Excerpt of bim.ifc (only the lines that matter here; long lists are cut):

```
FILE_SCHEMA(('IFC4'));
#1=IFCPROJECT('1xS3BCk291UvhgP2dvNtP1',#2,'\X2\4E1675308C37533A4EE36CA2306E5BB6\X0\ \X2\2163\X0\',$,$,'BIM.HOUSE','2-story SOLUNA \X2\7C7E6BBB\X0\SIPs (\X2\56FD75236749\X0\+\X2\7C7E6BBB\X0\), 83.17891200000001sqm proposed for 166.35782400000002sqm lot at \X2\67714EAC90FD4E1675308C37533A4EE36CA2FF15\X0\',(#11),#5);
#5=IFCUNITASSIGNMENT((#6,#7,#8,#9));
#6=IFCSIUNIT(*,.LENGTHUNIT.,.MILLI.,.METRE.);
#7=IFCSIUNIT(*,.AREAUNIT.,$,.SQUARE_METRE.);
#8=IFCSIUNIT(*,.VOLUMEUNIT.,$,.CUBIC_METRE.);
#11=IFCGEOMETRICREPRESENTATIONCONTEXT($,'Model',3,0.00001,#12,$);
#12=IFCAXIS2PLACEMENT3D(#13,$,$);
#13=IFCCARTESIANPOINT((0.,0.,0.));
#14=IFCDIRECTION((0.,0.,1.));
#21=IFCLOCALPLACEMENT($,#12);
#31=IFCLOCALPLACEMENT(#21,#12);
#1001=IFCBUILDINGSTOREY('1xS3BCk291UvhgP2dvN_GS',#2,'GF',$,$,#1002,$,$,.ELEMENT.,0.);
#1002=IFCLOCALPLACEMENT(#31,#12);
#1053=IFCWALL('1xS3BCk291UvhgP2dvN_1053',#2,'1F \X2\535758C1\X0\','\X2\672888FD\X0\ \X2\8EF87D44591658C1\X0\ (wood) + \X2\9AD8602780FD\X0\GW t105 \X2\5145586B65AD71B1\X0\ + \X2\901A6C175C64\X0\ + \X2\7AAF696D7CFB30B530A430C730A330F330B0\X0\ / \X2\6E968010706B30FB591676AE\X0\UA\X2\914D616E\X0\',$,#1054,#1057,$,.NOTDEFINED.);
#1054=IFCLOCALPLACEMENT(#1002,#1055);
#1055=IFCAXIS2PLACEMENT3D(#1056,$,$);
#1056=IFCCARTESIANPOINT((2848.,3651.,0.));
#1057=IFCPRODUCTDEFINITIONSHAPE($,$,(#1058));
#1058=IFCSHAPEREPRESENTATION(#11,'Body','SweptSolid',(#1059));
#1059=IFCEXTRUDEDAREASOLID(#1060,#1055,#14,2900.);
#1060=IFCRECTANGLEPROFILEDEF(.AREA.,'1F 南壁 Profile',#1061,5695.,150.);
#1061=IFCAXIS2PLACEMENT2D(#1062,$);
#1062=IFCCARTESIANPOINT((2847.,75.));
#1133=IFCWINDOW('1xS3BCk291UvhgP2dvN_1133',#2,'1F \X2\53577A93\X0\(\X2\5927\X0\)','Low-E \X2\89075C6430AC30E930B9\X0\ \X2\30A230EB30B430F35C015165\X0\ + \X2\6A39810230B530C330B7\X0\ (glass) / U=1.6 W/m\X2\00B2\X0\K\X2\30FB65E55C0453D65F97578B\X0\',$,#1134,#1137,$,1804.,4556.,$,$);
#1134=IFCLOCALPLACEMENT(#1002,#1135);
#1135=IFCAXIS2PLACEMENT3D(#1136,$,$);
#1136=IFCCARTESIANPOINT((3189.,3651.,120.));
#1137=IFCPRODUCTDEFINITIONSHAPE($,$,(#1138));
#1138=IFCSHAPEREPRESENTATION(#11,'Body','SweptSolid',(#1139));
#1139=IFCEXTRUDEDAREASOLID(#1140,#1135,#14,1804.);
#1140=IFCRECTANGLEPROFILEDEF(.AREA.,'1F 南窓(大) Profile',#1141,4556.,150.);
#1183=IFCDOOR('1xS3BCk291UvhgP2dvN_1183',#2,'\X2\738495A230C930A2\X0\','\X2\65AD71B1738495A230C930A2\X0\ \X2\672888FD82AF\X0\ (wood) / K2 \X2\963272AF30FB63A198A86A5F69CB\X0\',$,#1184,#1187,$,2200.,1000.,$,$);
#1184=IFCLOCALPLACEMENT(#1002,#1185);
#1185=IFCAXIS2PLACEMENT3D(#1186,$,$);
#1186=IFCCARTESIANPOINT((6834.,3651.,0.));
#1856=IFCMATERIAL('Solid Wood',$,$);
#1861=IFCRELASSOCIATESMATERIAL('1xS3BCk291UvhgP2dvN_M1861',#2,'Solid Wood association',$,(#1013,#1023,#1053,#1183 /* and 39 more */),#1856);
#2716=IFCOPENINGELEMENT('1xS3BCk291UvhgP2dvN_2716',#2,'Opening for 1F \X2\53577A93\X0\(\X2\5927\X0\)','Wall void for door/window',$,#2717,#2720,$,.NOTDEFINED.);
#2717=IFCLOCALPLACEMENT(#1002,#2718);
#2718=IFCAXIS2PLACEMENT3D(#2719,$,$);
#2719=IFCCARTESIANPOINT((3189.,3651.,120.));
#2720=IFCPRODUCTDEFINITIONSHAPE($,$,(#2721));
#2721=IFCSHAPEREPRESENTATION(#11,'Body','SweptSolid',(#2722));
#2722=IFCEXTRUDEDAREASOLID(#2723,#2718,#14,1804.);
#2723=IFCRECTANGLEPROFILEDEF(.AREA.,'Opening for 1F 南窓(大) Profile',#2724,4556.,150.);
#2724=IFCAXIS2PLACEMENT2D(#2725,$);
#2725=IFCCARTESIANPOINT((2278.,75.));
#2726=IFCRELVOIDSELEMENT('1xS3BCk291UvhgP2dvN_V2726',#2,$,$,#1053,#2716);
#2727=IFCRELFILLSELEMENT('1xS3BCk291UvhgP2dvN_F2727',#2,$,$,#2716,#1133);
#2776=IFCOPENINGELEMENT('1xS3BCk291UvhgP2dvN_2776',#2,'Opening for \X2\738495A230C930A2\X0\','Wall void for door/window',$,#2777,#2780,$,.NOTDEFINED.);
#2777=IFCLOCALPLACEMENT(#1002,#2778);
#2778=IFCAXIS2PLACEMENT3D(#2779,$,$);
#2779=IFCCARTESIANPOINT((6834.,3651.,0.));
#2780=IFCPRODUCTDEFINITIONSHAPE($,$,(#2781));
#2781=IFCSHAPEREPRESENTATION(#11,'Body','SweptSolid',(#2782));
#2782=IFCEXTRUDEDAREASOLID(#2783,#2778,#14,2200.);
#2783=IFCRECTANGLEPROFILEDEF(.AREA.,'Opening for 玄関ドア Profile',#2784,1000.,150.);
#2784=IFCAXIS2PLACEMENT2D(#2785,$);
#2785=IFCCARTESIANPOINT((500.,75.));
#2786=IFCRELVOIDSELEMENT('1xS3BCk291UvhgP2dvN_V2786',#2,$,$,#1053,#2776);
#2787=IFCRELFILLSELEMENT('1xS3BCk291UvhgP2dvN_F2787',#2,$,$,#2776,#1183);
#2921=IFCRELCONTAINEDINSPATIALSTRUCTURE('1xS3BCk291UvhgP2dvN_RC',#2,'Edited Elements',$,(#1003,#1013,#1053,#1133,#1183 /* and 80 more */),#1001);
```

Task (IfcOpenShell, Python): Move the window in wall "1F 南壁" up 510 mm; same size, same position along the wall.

```python
import numpy as np
import ifcopenshell
import ifcopenshell.api.geometry
import ifcopenshell.util.placement
import ifcopenshell.util.unit

model = ifcopenshell.open("bim.ifc")
unit_scale = ifcopenshell.util.unit.calculate_unit_scale(model)

window = model.by_id(1133)
opening = window.FillsVoids[0].RelatingOpeningElement
dz = 0.51 / unit_scale

shift = np.array([0.0, 0.0, dz])
# The window is not placed relative to its opening, so move both.
for product in (opening, window):
    matrix = ifcopenshell.util.placement.get_local_placement(product.ObjectPlacement)
    matrix[:3, 3] += shift
    ifcopenshell.api.geometry.edit_object_placement(model, product=product, matrix=matrix, is_si=False)

print(f"moved by {dz * unit_scale:+.3f} m")

model.write("bim_v2.ifc")
```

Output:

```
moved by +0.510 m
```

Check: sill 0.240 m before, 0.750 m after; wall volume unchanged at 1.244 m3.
